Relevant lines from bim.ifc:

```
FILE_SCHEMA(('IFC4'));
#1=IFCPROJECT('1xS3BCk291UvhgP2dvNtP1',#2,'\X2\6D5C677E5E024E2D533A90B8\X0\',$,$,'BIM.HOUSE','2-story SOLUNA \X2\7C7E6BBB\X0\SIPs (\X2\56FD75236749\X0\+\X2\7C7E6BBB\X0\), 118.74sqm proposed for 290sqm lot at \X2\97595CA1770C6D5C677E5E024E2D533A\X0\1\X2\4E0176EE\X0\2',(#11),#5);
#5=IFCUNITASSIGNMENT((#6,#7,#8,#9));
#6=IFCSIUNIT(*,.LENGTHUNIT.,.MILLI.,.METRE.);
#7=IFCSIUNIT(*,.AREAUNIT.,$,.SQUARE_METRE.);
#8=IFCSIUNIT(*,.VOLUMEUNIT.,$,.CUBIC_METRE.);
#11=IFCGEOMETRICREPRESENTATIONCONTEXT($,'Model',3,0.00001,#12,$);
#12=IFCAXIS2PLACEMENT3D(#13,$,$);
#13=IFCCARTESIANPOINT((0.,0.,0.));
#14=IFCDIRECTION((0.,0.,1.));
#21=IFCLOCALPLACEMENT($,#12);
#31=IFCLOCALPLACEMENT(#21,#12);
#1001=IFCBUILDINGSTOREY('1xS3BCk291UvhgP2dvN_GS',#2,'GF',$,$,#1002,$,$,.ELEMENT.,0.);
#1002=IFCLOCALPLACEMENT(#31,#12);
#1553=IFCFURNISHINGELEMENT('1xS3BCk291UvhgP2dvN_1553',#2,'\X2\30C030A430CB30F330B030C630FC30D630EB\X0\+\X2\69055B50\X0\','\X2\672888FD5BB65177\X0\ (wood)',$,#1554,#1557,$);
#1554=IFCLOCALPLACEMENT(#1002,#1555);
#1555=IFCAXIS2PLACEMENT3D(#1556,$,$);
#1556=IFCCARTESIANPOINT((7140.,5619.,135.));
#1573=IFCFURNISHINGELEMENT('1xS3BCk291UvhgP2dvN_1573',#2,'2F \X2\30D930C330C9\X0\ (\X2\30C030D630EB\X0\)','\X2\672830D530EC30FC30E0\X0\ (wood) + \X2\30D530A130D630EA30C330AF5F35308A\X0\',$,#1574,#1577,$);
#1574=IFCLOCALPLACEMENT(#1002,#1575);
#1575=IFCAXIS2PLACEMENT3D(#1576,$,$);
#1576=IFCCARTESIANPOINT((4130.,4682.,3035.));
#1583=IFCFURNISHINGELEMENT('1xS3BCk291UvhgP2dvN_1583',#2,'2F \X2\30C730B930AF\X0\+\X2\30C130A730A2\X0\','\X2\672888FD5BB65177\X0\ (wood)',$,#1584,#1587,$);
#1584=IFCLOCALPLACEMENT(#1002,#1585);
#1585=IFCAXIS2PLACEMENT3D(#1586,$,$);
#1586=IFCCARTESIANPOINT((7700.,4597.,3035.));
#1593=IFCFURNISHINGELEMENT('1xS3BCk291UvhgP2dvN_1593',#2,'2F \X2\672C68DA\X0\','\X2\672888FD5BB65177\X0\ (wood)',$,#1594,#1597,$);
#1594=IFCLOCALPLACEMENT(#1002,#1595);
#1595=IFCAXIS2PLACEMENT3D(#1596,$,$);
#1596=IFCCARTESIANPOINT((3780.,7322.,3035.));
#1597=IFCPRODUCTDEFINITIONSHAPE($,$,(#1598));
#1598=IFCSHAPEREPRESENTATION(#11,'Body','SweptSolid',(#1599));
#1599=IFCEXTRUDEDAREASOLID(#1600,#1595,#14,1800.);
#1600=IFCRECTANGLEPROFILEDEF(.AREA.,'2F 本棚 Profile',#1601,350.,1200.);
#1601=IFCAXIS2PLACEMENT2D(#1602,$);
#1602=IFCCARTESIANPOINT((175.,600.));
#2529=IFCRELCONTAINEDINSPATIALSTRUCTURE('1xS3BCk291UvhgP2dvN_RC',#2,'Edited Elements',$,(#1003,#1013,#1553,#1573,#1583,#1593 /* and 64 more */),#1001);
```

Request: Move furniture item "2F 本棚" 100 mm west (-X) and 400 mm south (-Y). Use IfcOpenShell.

```python
import ifcopenshell
import ifcopenshell.api.geometry
import ifcopenshell.util.placement
import ifcopenshell.util.unit

model = ifcopenshell.open("bim.ifc")
unit_scale = ifcopenshell.util.unit.calculate_unit_scale(model)

item = model.by_guid("1xS3BCk291UvhgP2dvN_1593")
matrix = ifcopenshell.util.placement.get_local_placement(item.ObjectPlacement)
matrix[0, 3] -= 0.1 / unit_scale
matrix[1, 3] -= 0.4 / unit_scale
ifcopenshell.api.geometry.edit_object_placement(model, product=item, matrix=matrix, is_si=False)

print(ifcopenshell.util.placement.get_local_placement(item.ObjectPlacement).round(3) + 0.0)

model.write("bim_updated.ifc")
```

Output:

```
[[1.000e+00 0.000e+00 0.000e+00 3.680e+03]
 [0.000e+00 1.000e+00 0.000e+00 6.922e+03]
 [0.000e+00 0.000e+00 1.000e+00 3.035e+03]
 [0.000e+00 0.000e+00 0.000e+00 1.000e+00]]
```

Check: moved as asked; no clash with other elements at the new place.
